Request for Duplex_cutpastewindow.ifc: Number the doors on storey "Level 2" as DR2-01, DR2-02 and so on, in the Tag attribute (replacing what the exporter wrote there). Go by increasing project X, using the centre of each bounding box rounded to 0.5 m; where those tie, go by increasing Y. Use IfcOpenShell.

First a look at what the model holds.

```python
import ifcopenshell
import ifcopenshell.util.element
import ifcopenshell.util.placement

model = ifcopenshell.open("Duplex_cutpastewindow.ifc")
print(model.schema)
storey = next(s for s in model.by_type("IfcBuildingStorey") if s.Name == "Level 2")
doors = [e for e in ifcopenshell.util.element.get_decomposition(storey) if e.is_a("IfcDoor")]
for e in sorted(doors, key=lambda e: e.id()):
    origin = ifcopenshell.util.placement.get_local_placement(e.ObjectPlacement)[:3, 3]
    print(e.id(), e.Tag, e.Name, origin.round(2) + 0.0, sep=" | ")
```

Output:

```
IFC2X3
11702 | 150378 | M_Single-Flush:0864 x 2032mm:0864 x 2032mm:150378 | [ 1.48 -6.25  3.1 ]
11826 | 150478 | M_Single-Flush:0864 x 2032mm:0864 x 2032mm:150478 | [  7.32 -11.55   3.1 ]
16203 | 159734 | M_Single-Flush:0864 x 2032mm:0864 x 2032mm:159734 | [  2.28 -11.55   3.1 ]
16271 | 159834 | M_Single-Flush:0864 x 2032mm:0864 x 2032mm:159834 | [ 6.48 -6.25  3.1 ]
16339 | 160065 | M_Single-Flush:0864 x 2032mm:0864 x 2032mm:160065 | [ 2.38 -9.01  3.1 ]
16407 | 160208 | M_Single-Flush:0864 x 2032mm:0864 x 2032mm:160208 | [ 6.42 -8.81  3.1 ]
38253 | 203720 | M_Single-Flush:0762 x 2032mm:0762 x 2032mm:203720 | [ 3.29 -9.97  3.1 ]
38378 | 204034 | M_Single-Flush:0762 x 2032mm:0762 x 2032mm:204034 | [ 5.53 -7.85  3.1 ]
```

```python
import ifcopenshell
import ifcopenshell.geom
import ifcopenshell.util.element
import ifcopenshell.util.shape

model = ifcopenshell.open("Duplex_cutpastewindow.ifc")
settings = ifcopenshell.geom.settings()
settings.set("use-world-coords", True)


def centre(element):
    shape = ifcopenshell.geom.create_shape(settings, element)
    return ifcopenshell.util.shape.get_bbox_centroid(shape.geometry)


storey = next(s for s in model.by_type("IfcBuildingStorey") if s.Name == "Level 2")
doors = [e for e in ifcopenshell.util.element.get_decomposition(storey) if e.is_a("IfcDoor")]

# Insertion points can sit at a corner or the storey origin, so sort by the geometry (in metres).
centres = {e: centre(e) for e in doors}
doors.sort(key=lambda e: (round(centres[e][0] / 0.5), centres[e][1]))

for i, e in enumerate(doors, start=1):
    number = f"DR2-{i:02d}"
    e.Tag = number
    print(e.id(), number)

model.write("Duplex_cutpastewindow_edited.ifc")
```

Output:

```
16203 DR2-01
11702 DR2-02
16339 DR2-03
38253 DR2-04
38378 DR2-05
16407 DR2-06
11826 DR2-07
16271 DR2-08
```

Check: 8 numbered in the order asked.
